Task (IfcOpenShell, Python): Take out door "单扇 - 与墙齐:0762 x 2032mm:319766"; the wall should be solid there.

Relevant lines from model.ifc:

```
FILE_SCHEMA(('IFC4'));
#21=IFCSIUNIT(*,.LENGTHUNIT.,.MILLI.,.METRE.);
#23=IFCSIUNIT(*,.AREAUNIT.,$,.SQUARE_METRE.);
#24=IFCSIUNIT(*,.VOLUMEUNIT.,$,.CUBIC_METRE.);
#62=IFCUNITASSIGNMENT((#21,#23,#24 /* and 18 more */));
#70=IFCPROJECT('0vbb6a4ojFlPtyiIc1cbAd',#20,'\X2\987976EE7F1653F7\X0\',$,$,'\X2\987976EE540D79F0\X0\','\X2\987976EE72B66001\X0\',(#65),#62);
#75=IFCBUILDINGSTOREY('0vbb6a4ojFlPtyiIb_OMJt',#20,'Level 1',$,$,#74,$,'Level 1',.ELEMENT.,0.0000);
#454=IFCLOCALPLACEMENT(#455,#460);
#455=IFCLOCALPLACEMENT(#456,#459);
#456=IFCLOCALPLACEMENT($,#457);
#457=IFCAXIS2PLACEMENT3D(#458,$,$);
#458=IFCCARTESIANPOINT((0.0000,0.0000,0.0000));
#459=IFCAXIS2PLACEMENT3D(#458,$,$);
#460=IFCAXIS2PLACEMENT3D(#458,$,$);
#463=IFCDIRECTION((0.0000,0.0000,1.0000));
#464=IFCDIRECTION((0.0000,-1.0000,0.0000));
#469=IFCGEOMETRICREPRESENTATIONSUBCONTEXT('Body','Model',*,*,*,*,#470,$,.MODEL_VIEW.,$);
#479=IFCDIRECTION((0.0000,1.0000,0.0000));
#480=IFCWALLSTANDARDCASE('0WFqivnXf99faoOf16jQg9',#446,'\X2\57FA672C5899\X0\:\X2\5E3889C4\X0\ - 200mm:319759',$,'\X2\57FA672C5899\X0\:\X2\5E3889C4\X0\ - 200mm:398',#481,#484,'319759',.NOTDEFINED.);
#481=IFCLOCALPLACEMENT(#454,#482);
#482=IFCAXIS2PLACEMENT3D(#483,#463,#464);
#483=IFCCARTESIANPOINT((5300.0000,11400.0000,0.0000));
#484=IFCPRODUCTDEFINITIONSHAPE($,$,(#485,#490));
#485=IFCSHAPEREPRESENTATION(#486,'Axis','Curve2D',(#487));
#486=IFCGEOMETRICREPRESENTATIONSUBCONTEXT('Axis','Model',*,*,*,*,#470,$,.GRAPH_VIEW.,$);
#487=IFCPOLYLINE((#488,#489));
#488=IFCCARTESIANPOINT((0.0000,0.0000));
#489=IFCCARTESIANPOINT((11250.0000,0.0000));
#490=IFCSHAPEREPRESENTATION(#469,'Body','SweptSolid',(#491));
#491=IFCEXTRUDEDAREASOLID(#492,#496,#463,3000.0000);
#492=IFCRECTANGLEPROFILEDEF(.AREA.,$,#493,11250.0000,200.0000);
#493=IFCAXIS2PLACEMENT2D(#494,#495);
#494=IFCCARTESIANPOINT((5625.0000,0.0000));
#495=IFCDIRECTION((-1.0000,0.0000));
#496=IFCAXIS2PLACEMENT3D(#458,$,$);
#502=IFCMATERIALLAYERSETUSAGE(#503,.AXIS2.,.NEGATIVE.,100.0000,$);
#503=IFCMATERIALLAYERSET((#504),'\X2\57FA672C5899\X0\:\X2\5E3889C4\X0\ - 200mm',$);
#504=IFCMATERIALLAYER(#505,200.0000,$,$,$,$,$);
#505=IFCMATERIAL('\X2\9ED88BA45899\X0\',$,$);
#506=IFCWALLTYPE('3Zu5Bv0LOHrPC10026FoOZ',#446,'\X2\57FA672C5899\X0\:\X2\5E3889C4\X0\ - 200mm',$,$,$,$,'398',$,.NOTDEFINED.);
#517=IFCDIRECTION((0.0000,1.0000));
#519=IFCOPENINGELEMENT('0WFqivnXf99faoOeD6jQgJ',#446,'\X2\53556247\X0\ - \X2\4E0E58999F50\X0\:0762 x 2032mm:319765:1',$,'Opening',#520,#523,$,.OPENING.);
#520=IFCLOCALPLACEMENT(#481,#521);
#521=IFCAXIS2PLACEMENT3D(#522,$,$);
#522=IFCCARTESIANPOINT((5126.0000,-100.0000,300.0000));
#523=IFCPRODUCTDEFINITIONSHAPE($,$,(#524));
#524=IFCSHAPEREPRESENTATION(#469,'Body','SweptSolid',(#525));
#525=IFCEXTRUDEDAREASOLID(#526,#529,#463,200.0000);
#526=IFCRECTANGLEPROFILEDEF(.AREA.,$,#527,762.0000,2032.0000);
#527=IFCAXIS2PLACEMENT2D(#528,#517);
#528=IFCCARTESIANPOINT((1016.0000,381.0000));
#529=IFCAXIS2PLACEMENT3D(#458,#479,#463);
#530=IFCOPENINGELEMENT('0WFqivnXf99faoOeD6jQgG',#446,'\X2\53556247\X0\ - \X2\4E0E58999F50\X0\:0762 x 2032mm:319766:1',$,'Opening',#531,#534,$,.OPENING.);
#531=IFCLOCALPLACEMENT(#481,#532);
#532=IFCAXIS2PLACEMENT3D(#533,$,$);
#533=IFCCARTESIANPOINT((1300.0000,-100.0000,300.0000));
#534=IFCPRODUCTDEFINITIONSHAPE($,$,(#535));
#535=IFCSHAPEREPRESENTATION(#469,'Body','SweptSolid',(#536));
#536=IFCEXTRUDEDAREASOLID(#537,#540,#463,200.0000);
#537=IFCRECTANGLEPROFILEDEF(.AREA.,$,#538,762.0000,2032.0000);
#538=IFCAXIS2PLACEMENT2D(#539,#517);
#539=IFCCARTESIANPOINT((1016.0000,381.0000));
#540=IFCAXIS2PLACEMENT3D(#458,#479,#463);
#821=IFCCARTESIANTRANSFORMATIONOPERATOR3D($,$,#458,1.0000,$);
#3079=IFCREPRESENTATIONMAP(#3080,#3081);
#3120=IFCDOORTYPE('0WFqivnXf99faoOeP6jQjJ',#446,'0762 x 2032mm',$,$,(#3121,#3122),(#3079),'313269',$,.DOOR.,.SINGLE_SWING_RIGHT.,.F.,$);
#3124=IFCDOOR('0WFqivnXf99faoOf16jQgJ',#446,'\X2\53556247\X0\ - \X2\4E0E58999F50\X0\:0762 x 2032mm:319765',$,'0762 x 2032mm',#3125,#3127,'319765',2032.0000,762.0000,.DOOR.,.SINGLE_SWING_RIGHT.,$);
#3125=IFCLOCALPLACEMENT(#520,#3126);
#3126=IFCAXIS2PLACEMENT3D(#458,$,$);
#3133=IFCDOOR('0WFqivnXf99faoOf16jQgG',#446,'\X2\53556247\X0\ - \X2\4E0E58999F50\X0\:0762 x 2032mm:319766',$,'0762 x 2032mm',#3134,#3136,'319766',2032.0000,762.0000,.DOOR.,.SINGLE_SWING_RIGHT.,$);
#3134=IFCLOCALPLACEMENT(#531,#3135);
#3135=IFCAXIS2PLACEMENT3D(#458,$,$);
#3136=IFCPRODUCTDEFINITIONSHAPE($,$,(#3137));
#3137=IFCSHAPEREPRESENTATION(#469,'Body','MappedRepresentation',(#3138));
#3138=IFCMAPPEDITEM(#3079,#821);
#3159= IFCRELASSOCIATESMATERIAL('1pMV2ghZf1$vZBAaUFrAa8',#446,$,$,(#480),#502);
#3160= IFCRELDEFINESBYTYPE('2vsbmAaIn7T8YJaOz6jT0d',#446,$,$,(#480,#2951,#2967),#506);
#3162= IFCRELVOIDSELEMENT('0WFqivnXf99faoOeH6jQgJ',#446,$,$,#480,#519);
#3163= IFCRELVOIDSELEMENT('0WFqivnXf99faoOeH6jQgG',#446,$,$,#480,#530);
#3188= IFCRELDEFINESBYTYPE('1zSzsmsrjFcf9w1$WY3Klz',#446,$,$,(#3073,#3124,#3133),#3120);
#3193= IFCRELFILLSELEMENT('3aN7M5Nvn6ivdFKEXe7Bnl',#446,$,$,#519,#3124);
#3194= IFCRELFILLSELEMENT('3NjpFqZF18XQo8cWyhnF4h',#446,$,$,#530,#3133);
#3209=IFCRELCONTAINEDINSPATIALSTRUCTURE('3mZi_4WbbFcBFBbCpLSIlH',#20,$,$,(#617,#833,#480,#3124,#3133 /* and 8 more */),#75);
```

```python
import ifcopenshell
import ifcopenshell.api.feature
import ifcopenshell.api.root
import ifcopenshell.geom
import ifcopenshell.util.shape

model = ifcopenshell.open("model.ifc")
settings = ifcopenshell.geom.settings()


def volume(element):
    """Net volume in cubic metres, openings subtracted."""
    shape = ifcopenshell.geom.create_shape(settings, element)
    return ifcopenshell.util.shape.get_volume(shape.geometry)


door = model.by_guid("0WFqivnXf99faoOf16jQgG")
opening = door.FillsVoids[0].RelatingOpeningElement
wall = opening.VoidsElements[0].RelatingBuildingElement
before = volume(wall)

ifcopenshell.api.root.remove_product(model, product=door)
ifcopenshell.api.feature.remove_feature(model, feature=opening)

after = volume(wall)

print(f"wall volume {before:.3f} -> {after:.3f} m3")

model.write("model_updated.ifc")
```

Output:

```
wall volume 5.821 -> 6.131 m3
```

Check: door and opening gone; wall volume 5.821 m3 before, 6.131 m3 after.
